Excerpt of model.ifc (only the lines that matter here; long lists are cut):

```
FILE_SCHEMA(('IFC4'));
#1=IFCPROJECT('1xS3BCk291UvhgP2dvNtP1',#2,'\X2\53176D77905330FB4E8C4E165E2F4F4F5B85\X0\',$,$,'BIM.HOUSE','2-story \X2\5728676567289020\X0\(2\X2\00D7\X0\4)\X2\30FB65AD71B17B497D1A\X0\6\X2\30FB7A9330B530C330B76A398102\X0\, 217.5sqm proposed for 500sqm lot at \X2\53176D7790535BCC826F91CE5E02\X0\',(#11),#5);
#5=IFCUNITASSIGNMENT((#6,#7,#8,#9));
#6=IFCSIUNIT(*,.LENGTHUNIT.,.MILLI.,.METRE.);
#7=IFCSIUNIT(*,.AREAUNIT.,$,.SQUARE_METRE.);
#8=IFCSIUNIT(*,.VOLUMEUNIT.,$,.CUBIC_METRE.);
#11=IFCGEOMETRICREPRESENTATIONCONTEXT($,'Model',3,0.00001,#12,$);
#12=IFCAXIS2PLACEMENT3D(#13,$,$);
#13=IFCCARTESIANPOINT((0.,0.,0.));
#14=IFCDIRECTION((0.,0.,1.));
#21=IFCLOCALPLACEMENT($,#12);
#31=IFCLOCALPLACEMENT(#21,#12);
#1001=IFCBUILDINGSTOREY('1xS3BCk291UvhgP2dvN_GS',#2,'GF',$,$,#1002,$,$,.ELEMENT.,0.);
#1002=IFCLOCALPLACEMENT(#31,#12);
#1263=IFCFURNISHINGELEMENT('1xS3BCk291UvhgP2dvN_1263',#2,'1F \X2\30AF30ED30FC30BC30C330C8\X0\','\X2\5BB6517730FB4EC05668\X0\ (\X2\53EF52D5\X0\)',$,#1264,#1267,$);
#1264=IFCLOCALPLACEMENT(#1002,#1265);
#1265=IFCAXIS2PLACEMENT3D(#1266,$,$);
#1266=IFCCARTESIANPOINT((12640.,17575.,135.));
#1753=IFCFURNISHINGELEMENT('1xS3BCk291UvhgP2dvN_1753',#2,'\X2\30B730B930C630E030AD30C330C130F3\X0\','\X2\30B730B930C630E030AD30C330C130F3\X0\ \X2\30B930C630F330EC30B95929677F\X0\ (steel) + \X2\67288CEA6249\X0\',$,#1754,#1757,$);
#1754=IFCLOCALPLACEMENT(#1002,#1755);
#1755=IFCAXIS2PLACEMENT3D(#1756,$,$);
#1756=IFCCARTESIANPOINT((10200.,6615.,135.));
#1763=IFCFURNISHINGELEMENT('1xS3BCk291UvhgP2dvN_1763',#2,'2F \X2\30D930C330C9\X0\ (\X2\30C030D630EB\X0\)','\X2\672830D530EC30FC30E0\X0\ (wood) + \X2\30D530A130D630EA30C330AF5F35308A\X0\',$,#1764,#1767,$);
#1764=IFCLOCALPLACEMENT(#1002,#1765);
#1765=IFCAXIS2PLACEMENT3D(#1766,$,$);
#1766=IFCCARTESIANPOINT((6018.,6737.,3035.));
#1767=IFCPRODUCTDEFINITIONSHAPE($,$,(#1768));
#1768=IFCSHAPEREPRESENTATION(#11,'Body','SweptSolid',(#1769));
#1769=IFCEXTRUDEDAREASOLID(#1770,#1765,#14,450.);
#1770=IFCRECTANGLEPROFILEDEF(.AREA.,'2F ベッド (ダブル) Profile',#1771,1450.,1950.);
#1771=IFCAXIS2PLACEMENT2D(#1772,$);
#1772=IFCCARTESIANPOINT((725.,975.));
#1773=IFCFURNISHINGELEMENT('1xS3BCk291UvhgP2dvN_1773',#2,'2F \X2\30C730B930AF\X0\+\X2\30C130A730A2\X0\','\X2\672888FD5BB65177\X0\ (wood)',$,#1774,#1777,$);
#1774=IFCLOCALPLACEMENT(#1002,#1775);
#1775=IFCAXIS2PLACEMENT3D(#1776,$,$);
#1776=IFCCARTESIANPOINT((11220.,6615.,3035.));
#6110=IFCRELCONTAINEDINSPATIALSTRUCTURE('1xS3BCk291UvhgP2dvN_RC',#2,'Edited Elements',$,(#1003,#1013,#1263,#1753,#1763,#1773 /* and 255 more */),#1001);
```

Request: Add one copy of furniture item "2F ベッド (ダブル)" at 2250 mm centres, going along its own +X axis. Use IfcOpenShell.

```python
import ifcopenshell
import ifcopenshell.api.geometry
import ifcopenshell.api.root
import ifcopenshell.util.element
import ifcopenshell.util.placement

model = ifcopenshell.open("model.ifc")


def reuse_history(source, copy):
    """copy_class also copies each property set's owner history, people and application; keep the originals."""
    for rel in copy.IsDefinedBy:
        if rel.is_a("IfcRelDefinesByProperties") and (history := rel.RelatingPropertyDefinition.OwnerHistory):
            rel.RelatingPropertyDefinition.OwnerHistory = source.OwnerHistory
            ifcopenshell.util.element.remove_deep2(model, history)


source = model.by_guid("1xS3BCk291UvhgP2dvN_1763")
base = ifcopenshell.util.placement.get_local_placement(source.ObjectPlacement)
step = base[:3, 0] * 2250.0

for i in range(1, 2):
    copy = ifcopenshell.api.root.copy_class(model, product=source)
    copy.Representation = ifcopenshell.util.element.copy_deep(
        model, source.Representation, exclude=["IfcGeometricRepresentationContext", "IfcRepresentationMap"]
    )
    reuse_history(source, copy)
    matrix = base.copy()
    matrix[:3, 3] += i * step
    print("added at", matrix[:3, 3].round(3) + 0.0)
    ifcopenshell.api.geometry.edit_object_placement(model, product=copy, matrix=matrix, is_si=False)

model.write("model_v2.ifc")
```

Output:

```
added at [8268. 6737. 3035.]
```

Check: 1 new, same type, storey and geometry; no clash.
